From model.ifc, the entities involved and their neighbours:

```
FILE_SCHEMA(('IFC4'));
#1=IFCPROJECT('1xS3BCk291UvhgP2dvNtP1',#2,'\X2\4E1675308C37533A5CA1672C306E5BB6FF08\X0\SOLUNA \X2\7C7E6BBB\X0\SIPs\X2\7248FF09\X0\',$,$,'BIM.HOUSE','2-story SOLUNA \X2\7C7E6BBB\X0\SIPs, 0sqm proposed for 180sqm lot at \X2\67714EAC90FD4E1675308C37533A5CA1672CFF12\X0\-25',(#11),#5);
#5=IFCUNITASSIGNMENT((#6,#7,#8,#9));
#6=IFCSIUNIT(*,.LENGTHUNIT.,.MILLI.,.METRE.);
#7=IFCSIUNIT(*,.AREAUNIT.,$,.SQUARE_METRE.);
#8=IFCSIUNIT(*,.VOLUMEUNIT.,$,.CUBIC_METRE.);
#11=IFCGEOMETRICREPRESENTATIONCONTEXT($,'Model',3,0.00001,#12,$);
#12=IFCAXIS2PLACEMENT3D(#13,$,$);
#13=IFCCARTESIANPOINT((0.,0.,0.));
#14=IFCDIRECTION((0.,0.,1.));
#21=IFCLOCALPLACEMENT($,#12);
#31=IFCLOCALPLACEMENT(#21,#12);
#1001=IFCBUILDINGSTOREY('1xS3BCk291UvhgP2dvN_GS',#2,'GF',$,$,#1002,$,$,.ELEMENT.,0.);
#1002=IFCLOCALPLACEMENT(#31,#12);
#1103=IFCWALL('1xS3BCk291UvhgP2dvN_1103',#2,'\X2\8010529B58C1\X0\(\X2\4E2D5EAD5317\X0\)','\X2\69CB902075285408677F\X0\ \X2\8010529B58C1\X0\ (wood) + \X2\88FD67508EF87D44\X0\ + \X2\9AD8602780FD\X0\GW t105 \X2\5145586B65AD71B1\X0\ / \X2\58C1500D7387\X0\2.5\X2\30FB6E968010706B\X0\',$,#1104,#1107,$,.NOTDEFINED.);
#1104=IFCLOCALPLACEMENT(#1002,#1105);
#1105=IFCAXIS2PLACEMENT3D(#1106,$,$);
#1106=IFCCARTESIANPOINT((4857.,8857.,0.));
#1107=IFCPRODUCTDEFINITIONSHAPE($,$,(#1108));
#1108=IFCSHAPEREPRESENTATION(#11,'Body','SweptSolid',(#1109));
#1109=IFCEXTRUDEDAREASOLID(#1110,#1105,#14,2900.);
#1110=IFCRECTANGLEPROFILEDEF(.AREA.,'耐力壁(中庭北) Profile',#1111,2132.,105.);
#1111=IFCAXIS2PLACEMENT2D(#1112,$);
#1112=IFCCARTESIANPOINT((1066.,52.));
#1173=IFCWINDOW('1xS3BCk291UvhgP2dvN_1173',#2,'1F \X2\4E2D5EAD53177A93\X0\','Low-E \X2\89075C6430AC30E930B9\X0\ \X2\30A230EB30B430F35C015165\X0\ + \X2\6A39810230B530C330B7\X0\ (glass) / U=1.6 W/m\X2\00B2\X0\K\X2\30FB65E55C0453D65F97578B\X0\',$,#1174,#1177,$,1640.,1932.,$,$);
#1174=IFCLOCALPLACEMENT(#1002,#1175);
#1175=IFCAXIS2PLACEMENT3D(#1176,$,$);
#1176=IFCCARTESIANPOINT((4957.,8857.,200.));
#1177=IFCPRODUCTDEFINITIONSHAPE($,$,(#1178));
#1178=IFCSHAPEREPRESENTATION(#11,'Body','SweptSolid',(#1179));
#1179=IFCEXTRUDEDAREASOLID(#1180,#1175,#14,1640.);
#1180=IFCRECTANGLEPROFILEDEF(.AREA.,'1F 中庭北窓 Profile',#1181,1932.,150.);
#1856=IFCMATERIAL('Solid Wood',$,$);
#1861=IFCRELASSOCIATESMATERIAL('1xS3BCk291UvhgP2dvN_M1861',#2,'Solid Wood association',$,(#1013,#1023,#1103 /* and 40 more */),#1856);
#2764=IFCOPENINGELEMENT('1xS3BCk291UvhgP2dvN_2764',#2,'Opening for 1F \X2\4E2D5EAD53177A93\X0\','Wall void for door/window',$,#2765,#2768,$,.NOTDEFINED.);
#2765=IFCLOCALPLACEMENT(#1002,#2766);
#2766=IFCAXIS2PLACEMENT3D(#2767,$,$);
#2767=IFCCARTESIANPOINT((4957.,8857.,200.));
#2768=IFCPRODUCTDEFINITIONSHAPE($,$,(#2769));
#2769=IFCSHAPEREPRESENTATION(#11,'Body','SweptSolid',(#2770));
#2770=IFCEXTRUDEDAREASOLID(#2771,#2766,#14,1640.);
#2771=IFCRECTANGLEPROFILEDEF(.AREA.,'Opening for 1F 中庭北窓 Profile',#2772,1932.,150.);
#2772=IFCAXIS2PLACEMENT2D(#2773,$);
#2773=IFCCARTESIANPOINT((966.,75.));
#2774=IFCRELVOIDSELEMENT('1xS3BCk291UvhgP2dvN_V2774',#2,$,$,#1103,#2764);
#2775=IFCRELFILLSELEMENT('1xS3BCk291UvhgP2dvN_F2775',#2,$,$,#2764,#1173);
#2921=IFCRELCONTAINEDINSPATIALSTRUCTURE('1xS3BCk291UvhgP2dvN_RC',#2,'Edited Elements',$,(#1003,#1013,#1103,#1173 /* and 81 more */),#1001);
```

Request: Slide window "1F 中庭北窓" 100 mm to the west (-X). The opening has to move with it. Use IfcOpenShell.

```python
import ifcopenshell
import ifcopenshell.api.geometry
import ifcopenshell.util.placement
import ifcopenshell.util.unit

model = ifcopenshell.open("model.ifc")
unit_scale = ifcopenshell.util.unit.calculate_unit_scale(model)

window = model.by_guid("1xS3BCk291UvhgP2dvN_1173")
opening = window.FillsVoids[0].RelatingOpeningElement
wall = opening.VoidsElements[0].RelatingBuildingElement

wall_matrix = ifcopenshell.util.placement.get_local_placement(wall.ObjectPlacement)
shift = wall_matrix[:3, 0] * -0.1 / unit_scale
before = ifcopenshell.util.placement.get_local_placement(window.ObjectPlacement)[:3, 3].copy()

# The window is not placed relative to its opening, so move both.
for product in (opening, window):
    matrix = ifcopenshell.util.placement.get_local_placement(product.ObjectPlacement)
    matrix[:3, 3] += shift
    ifcopenshell.api.geometry.edit_object_placement(model, product=product, matrix=matrix, is_si=False)

after = ifcopenshell.util.placement.get_local_placement(window.ObjectPlacement)[:3, 3]
print("window moved by", (after - before).round(3) + 0.0)

model.write("model_rev.ifc")
```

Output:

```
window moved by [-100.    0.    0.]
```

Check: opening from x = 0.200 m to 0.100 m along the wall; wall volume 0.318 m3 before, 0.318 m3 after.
